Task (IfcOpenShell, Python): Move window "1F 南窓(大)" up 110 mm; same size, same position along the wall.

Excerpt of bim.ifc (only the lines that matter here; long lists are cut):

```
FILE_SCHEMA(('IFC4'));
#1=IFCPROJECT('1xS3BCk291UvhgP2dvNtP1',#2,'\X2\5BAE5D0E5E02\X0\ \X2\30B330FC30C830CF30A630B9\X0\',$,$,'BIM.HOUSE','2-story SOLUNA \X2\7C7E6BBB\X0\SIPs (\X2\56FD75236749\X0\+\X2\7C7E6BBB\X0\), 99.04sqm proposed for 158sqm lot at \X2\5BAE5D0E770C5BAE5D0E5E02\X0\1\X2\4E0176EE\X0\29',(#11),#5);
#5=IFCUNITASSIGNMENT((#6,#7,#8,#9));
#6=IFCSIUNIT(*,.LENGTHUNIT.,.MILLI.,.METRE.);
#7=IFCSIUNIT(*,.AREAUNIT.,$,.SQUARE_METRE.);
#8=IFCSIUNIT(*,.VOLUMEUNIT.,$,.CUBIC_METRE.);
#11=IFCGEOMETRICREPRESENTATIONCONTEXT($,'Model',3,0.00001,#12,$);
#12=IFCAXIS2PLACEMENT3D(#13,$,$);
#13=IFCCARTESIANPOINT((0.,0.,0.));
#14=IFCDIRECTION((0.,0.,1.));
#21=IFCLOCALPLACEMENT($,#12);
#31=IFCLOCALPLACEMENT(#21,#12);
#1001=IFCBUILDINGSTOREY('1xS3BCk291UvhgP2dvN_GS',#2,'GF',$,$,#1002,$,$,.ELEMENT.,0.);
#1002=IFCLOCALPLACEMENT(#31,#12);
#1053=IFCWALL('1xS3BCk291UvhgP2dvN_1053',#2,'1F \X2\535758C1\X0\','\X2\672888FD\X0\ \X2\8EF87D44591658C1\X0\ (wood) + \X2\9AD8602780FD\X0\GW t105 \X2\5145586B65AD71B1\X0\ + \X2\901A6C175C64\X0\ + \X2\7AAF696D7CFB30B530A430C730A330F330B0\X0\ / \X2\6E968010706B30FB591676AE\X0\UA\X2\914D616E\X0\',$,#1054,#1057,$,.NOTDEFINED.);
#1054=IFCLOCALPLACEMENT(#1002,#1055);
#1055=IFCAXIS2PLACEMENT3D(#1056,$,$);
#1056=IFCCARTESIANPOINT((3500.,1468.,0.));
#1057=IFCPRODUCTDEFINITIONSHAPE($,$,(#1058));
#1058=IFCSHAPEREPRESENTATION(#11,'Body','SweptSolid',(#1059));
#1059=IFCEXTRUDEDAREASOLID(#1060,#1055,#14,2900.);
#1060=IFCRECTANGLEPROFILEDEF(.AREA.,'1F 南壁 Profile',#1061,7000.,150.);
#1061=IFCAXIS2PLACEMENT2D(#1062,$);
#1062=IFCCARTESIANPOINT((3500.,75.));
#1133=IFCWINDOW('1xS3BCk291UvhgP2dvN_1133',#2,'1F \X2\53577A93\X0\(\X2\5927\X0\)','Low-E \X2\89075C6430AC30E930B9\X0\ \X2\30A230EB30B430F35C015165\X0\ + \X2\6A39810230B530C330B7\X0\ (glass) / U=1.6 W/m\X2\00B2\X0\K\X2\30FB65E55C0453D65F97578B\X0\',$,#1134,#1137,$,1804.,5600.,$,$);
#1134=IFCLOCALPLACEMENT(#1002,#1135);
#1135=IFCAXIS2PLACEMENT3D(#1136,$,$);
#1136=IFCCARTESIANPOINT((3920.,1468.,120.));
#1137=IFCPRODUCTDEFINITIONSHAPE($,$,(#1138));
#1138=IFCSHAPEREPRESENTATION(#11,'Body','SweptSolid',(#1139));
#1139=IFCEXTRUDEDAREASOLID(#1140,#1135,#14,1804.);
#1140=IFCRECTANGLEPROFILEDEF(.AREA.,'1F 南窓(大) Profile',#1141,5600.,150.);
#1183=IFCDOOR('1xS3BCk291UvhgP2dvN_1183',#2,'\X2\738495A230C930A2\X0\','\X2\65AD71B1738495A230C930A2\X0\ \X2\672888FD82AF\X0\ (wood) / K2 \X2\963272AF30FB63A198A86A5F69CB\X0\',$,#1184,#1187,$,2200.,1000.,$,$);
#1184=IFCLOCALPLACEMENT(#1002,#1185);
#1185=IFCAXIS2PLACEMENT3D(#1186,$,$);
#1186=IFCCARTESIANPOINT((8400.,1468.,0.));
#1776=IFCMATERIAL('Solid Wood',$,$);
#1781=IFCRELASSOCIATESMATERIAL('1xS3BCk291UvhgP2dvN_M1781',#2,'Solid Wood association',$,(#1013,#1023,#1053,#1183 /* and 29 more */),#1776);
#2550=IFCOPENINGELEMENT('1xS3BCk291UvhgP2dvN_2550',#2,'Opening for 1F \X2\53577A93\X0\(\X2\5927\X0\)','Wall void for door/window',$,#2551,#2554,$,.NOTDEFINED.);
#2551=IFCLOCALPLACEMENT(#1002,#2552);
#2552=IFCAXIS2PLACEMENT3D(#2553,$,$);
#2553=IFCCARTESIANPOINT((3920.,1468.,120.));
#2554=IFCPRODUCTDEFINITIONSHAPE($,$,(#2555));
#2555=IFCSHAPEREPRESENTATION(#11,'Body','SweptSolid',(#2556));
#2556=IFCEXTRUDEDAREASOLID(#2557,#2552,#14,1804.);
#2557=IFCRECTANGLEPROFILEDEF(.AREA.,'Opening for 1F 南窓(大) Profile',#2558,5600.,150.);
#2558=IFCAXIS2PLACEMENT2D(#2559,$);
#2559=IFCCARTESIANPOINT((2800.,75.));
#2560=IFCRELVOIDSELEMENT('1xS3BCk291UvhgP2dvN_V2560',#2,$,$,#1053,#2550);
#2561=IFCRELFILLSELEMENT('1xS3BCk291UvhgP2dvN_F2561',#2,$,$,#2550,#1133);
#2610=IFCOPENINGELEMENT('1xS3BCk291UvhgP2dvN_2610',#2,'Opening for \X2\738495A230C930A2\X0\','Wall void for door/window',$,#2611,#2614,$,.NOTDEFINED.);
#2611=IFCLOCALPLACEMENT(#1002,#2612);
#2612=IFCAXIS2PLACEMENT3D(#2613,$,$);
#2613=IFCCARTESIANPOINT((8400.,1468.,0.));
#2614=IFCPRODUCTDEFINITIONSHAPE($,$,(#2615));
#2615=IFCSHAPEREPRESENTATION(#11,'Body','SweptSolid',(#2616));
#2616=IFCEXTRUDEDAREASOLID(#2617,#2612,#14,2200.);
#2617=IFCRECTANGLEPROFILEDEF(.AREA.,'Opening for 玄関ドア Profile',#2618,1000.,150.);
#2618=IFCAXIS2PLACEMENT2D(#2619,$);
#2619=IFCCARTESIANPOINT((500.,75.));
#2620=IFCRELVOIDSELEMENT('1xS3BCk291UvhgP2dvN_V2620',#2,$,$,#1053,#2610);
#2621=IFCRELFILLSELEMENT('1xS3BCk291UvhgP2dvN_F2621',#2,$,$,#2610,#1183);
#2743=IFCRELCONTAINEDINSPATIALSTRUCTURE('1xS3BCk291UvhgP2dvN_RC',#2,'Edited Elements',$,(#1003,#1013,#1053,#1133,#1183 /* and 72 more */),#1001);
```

```python
import numpy as np
import ifcopenshell
import ifcopenshell.api.geometry
import ifcopenshell.util.placement
import ifcopenshell.util.unit

model = ifcopenshell.open("bim.ifc")
unit_scale = ifcopenshell.util.unit.calculate_unit_scale(model)

window = model.by_guid("1xS3BCk291UvhgP2dvN_1133")
opening = window.FillsVoids[0].RelatingOpeningElement
dz = 0.11 / unit_scale

shift = np.array([0.0, 0.0, dz])
# The window is not placed relative to its opening, so move both.
for product in (opening, window):
    matrix = ifcopenshell.util.placement.get_local_placement(product.ObjectPlacement)
    matrix[:3, 3] += shift
    ifcopenshell.api.geometry.edit_object_placement(model, product=product, matrix=matrix, is_si=False)

print(f"moved by {dz * unit_scale:+.3f} m")

model.write("bim_rev.ifc")
```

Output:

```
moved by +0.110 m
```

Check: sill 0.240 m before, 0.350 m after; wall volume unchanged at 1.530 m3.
